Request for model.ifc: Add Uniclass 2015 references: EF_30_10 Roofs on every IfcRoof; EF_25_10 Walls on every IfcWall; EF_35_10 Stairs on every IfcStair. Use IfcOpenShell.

First a look at what the model holds.

```python
import ifcopenshell

model = ifcopenshell.open("model.ifc")
print(model.schema)
print("classifications:", [c.Name for c in model.by_type("IfcClassification")])
for ifc_class in ("IfcDoor", "IfcRoof", "IfcStair", "IfcWall", "IfcWindow"):
    print(ifc_class, len(model.by_type(ifc_class)))
```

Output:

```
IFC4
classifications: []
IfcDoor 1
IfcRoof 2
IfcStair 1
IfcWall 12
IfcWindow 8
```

```python
import ifcopenshell
import ifcopenshell.api.classification

model = ifcopenshell.open("model.ifc")

system = ifcopenshell.api.classification.add_classification(model, classification="Uniclass 2015")

codes = {
    "IfcRoof": ("EF_30_10", "Roofs"),
    "IfcWall": ("EF_25_10", "Walls"),
    "IfcStair": ("EF_35_10", "Stairs"),
}
for ifc_class, (code, name) in codes.items():
    products = model.by_type(ifc_class)
    ifcopenshell.api.classification.add_reference(
        model, products=products, classification=system, identification=code, name=name
    )
    print(code, len(products))

model.write("model_updated.ifc")
```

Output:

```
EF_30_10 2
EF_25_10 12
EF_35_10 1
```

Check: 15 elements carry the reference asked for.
